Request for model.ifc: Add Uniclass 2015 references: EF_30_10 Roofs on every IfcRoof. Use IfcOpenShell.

First a look at what the model holds.

```python
import ifcopenshell

model = ifcopenshell.open("model.ifc")
print(model.schema)
print("classifications:", [c.Name for c in model.by_type("IfcClassification")])
for ifc_class in ("IfcDoor", "IfcRoof", "IfcStair", "IfcWall", "IfcWindow"):
    print(ifc_class, len(model.by_type(ifc_class)))
```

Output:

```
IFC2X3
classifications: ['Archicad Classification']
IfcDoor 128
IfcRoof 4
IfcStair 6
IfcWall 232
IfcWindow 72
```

```python
import ifcopenshell
import ifcopenshell.api.classification

model = ifcopenshell.open("model.ifc")

# IFC2X3 requires Source and Edition and has no link from the project to the system.
system = model.create_entity("IfcClassification", Source="NBS", Edition="2015", Name="Uniclass 2015")

codes = {
    "IfcRoof": ("EF_30_10", "Roofs"),
}
for ifc_class, (code, name) in codes.items():
    products = model.by_type(ifc_class)
    ifcopenshell.api.classification.add_reference(
        model, products=products, classification=system, identification=code, name=name
    )
    print(code, len(products))

model.write("model_edited.ifc")
```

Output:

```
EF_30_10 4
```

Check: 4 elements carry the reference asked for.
